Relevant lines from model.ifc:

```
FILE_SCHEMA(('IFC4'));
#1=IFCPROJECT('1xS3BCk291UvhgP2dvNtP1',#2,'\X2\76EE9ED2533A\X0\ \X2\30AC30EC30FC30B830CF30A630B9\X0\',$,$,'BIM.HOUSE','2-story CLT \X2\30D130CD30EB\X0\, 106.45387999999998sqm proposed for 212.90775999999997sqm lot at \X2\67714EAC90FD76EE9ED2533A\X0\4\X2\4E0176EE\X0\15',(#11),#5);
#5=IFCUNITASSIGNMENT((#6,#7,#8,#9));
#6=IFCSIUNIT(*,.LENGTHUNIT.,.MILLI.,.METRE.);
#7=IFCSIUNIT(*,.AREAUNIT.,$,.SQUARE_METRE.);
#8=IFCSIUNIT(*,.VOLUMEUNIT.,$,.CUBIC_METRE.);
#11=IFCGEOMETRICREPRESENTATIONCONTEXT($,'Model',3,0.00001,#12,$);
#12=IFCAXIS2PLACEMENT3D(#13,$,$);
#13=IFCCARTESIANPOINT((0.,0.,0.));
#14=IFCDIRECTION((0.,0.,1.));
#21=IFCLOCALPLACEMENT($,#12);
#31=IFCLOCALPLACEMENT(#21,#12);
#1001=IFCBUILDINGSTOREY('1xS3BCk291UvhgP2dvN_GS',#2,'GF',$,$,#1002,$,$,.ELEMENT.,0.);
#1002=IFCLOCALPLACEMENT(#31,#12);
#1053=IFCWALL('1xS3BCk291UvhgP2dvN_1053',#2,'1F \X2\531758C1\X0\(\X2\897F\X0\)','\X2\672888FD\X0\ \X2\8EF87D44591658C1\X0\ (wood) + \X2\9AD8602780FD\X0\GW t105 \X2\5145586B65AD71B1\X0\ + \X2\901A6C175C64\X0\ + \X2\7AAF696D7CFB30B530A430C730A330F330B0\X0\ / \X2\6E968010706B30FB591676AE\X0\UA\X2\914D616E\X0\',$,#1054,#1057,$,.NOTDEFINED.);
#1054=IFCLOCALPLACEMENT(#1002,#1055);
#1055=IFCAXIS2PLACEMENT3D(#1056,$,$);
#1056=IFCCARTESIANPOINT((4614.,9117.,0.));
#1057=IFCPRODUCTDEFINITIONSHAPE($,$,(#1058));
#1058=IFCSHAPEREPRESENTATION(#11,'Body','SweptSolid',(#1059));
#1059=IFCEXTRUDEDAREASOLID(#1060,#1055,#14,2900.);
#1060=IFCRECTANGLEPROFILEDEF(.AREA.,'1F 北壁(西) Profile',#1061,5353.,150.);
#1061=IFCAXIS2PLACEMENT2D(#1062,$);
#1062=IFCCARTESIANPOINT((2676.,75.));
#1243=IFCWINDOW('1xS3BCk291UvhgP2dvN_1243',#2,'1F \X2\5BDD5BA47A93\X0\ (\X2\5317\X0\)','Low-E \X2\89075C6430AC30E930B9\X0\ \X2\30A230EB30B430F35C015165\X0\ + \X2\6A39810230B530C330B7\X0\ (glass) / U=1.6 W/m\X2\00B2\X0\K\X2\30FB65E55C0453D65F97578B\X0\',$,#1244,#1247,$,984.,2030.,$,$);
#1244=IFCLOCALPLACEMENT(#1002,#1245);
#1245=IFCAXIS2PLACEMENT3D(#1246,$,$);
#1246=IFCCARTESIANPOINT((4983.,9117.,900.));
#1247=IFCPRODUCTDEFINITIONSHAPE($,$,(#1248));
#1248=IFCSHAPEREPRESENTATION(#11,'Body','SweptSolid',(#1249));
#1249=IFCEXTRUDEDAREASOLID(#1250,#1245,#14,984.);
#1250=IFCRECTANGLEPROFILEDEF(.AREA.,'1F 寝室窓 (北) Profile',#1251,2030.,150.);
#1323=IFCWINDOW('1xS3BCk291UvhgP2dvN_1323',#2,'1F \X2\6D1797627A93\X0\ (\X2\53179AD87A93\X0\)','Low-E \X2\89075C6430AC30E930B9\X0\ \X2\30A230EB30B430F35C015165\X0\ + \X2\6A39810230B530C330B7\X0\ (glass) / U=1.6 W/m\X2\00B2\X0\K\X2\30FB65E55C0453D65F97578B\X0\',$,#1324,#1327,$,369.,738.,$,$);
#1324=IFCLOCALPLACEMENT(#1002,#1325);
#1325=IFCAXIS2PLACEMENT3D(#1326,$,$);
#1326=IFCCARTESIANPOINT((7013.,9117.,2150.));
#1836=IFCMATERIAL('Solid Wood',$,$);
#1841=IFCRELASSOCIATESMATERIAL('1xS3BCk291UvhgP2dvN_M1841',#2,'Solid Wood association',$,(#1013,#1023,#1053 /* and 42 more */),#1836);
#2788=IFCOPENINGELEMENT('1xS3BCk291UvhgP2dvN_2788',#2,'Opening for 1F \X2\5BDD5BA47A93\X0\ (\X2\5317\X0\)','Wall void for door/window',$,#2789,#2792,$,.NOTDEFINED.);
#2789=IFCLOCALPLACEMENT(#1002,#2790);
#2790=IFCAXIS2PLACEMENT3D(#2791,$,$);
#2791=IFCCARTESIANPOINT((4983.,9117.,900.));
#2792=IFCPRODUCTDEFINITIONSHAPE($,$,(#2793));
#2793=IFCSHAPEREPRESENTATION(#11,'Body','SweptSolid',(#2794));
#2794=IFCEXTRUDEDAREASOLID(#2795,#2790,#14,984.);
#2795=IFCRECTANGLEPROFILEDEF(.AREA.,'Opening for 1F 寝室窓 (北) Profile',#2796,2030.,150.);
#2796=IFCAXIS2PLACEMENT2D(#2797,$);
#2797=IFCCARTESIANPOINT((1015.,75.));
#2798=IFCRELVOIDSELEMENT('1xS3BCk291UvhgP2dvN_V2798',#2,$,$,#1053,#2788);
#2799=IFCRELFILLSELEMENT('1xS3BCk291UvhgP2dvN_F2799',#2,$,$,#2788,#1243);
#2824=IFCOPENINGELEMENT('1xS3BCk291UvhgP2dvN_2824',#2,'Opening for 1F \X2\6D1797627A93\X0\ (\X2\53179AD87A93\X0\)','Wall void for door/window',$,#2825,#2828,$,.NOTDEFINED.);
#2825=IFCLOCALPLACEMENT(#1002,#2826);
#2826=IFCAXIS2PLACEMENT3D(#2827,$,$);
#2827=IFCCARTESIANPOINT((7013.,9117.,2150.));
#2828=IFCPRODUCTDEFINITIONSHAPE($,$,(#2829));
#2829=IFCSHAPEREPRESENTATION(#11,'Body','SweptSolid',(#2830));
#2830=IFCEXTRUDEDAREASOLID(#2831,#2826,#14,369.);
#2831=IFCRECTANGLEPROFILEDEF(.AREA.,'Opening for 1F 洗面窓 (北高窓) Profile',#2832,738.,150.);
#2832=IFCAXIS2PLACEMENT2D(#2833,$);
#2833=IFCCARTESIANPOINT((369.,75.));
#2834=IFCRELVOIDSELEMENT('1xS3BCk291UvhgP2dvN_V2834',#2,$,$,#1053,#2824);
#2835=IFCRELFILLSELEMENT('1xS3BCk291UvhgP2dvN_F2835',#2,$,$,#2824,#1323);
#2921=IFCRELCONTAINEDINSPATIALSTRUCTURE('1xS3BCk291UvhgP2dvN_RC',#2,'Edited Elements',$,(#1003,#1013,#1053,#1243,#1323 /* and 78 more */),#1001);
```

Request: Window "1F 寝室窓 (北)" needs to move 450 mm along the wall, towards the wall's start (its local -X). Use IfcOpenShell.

```python
import ifcopenshell
import ifcopenshell.api.geometry
import ifcopenshell.util.placement
import ifcopenshell.util.unit

model = ifcopenshell.open("model.ifc")
unit_scale = ifcopenshell.util.unit.calculate_unit_scale(model)

window = model.by_guid("1xS3BCk291UvhgP2dvN_1243")
opening = window.FillsVoids[0].RelatingOpeningElement
wall = opening.VoidsElements[0].RelatingBuildingElement

wall_matrix = ifcopenshell.util.placement.get_local_placement(wall.ObjectPlacement)
shift = wall_matrix[:3, 0] * -0.45 / unit_scale
before = ifcopenshell.util.placement.get_local_placement(window.ObjectPlacement)[:3, 3].copy()

# The window is not placed relative to its opening, so move both.
for product in (opening, window):
    matrix = ifcopenshell.util.placement.get_local_placement(product.ObjectPlacement)
    matrix[:3, 3] += shift
    ifcopenshell.api.geometry.edit_object_placement(model, product=product, matrix=matrix, is_si=False)

after = ifcopenshell.util.placement.get_local_placement(window.ObjectPlacement)[:3, 3]
print("window moved by", (after - before).round(3) + 0.0)

model.write("model_edited.ifc")
```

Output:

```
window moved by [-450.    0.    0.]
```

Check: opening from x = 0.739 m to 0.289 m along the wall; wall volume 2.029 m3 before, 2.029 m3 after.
